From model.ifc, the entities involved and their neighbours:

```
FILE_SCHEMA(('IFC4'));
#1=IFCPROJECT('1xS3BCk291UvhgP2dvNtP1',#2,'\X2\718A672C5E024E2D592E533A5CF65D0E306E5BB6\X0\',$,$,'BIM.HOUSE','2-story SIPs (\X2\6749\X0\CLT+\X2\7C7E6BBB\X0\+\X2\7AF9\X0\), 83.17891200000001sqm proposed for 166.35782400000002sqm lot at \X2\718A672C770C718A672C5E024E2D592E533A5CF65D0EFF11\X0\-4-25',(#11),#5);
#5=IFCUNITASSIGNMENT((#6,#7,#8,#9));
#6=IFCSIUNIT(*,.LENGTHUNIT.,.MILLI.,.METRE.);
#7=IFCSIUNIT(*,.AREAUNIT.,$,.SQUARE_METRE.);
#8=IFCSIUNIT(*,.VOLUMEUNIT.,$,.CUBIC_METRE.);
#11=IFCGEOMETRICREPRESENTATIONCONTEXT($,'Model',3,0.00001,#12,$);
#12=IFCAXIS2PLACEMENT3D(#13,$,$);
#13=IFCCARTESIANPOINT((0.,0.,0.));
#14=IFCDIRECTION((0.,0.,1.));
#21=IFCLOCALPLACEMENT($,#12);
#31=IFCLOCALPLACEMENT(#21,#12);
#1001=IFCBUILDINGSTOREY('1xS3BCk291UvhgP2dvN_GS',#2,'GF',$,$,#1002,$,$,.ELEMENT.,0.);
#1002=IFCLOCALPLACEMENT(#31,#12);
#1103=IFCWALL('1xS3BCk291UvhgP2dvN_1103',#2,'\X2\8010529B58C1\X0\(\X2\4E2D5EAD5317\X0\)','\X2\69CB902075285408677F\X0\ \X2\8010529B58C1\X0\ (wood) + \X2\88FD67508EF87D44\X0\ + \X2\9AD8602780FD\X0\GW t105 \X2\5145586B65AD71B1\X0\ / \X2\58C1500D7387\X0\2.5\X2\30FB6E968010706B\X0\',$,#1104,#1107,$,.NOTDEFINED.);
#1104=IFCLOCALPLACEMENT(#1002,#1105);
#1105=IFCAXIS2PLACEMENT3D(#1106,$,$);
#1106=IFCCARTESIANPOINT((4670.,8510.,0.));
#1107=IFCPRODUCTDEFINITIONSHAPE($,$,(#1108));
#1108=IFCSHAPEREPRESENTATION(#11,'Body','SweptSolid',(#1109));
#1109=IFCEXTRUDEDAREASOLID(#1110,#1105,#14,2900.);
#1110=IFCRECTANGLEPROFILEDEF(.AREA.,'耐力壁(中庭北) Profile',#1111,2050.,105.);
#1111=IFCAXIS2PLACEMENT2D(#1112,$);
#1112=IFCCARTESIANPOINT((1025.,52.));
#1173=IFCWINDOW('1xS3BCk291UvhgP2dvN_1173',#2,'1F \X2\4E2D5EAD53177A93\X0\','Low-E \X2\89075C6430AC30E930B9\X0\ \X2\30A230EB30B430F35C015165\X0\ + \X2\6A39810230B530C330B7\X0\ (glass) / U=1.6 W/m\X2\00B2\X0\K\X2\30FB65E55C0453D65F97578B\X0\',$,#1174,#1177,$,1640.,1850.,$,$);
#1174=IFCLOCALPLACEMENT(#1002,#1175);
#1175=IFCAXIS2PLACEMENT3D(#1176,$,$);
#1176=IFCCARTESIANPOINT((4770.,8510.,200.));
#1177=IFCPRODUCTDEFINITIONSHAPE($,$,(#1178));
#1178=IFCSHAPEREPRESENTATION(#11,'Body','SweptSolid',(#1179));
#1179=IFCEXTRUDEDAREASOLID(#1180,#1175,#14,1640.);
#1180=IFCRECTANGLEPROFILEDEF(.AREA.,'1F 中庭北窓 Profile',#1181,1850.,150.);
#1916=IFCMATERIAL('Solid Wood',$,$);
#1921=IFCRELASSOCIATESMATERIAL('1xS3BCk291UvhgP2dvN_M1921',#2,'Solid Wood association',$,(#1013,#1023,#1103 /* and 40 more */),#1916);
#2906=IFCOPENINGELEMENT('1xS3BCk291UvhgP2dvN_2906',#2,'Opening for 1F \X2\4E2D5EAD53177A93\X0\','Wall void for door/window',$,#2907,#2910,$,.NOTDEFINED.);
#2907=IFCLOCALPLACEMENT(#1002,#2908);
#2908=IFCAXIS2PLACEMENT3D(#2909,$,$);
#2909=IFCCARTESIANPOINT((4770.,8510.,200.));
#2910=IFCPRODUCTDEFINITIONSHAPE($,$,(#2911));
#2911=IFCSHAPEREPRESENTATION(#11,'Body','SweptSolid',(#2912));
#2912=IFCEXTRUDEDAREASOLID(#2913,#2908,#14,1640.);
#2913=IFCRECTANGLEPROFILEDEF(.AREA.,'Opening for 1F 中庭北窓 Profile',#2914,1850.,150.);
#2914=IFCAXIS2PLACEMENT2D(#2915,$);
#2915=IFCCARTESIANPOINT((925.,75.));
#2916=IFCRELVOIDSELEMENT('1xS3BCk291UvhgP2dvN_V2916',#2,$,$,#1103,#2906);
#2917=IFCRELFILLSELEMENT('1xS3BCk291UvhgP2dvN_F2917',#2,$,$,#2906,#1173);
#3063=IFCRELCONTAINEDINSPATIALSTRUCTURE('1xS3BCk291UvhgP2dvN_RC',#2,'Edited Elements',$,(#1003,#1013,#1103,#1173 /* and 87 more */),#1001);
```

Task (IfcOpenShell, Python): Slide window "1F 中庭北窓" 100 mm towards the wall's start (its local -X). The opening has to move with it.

```python
import ifcopenshell
import ifcopenshell.api.geometry
import ifcopenshell.util.placement
import ifcopenshell.util.unit

model = ifcopenshell.open("model.ifc")
unit_scale = ifcopenshell.util.unit.calculate_unit_scale(model)

window = model.by_guid("1xS3BCk291UvhgP2dvN_1173")
opening = window.FillsVoids[0].RelatingOpeningElement
wall = opening.VoidsElements[0].RelatingBuildingElement

wall_matrix = ifcopenshell.util.placement.get_local_placement(wall.ObjectPlacement)
shift = wall_matrix[:3, 0] * -0.1 / unit_scale
before = ifcopenshell.util.placement.get_local_placement(window.ObjectPlacement)[:3, 3].copy()

# The window is not placed relative to its opening, so move both.
for product in (opening, window):
    matrix = ifcopenshell.util.placement.get_local_placement(product.ObjectPlacement)
    matrix[:3, 3] += shift
    ifcopenshell.api.geometry.edit_object_placement(model, product=product, matrix=matrix, is_si=False)

after = ifcopenshell.util.placement.get_local_placement(window.ObjectPlacement)[:3, 3]
print("window moved by", (after - before).round(3) + 0.0)

model.write("model_v2.ifc")
```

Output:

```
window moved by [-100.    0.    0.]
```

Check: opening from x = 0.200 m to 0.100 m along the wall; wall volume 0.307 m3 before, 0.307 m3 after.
